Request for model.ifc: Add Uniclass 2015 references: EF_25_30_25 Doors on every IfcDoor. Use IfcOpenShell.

First a look at what the model holds.

```python
import ifcopenshell

model = ifcopenshell.open("model.ifc")
print(model.schema)
print("classifications:", [c.Name for c in model.by_type("IfcClassification")])
for ifc_class in ("IfcDoor", "IfcRoof", "IfcStair", "IfcWall", "IfcWindow"):
    print(ifc_class, len(model.by_type(ifc_class)))
```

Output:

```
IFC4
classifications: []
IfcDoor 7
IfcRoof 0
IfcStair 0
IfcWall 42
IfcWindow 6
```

```python
import ifcopenshell
import ifcopenshell.api.classification

model = ifcopenshell.open("model.ifc")

system = ifcopenshell.api.classification.add_classification(model, classification="Uniclass 2015")

codes = {
    "IfcDoor": ("EF_25_30_25", "Doors"),
}
for ifc_class, (code, name) in codes.items():
    products = model.by_type(ifc_class)
    ifcopenshell.api.classification.add_reference(
        model, products=products, classification=system, identification=code, name=name
    )
    print(code, len(products))

model.write("model_edited.ifc")
```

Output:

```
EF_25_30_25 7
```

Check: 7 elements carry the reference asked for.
